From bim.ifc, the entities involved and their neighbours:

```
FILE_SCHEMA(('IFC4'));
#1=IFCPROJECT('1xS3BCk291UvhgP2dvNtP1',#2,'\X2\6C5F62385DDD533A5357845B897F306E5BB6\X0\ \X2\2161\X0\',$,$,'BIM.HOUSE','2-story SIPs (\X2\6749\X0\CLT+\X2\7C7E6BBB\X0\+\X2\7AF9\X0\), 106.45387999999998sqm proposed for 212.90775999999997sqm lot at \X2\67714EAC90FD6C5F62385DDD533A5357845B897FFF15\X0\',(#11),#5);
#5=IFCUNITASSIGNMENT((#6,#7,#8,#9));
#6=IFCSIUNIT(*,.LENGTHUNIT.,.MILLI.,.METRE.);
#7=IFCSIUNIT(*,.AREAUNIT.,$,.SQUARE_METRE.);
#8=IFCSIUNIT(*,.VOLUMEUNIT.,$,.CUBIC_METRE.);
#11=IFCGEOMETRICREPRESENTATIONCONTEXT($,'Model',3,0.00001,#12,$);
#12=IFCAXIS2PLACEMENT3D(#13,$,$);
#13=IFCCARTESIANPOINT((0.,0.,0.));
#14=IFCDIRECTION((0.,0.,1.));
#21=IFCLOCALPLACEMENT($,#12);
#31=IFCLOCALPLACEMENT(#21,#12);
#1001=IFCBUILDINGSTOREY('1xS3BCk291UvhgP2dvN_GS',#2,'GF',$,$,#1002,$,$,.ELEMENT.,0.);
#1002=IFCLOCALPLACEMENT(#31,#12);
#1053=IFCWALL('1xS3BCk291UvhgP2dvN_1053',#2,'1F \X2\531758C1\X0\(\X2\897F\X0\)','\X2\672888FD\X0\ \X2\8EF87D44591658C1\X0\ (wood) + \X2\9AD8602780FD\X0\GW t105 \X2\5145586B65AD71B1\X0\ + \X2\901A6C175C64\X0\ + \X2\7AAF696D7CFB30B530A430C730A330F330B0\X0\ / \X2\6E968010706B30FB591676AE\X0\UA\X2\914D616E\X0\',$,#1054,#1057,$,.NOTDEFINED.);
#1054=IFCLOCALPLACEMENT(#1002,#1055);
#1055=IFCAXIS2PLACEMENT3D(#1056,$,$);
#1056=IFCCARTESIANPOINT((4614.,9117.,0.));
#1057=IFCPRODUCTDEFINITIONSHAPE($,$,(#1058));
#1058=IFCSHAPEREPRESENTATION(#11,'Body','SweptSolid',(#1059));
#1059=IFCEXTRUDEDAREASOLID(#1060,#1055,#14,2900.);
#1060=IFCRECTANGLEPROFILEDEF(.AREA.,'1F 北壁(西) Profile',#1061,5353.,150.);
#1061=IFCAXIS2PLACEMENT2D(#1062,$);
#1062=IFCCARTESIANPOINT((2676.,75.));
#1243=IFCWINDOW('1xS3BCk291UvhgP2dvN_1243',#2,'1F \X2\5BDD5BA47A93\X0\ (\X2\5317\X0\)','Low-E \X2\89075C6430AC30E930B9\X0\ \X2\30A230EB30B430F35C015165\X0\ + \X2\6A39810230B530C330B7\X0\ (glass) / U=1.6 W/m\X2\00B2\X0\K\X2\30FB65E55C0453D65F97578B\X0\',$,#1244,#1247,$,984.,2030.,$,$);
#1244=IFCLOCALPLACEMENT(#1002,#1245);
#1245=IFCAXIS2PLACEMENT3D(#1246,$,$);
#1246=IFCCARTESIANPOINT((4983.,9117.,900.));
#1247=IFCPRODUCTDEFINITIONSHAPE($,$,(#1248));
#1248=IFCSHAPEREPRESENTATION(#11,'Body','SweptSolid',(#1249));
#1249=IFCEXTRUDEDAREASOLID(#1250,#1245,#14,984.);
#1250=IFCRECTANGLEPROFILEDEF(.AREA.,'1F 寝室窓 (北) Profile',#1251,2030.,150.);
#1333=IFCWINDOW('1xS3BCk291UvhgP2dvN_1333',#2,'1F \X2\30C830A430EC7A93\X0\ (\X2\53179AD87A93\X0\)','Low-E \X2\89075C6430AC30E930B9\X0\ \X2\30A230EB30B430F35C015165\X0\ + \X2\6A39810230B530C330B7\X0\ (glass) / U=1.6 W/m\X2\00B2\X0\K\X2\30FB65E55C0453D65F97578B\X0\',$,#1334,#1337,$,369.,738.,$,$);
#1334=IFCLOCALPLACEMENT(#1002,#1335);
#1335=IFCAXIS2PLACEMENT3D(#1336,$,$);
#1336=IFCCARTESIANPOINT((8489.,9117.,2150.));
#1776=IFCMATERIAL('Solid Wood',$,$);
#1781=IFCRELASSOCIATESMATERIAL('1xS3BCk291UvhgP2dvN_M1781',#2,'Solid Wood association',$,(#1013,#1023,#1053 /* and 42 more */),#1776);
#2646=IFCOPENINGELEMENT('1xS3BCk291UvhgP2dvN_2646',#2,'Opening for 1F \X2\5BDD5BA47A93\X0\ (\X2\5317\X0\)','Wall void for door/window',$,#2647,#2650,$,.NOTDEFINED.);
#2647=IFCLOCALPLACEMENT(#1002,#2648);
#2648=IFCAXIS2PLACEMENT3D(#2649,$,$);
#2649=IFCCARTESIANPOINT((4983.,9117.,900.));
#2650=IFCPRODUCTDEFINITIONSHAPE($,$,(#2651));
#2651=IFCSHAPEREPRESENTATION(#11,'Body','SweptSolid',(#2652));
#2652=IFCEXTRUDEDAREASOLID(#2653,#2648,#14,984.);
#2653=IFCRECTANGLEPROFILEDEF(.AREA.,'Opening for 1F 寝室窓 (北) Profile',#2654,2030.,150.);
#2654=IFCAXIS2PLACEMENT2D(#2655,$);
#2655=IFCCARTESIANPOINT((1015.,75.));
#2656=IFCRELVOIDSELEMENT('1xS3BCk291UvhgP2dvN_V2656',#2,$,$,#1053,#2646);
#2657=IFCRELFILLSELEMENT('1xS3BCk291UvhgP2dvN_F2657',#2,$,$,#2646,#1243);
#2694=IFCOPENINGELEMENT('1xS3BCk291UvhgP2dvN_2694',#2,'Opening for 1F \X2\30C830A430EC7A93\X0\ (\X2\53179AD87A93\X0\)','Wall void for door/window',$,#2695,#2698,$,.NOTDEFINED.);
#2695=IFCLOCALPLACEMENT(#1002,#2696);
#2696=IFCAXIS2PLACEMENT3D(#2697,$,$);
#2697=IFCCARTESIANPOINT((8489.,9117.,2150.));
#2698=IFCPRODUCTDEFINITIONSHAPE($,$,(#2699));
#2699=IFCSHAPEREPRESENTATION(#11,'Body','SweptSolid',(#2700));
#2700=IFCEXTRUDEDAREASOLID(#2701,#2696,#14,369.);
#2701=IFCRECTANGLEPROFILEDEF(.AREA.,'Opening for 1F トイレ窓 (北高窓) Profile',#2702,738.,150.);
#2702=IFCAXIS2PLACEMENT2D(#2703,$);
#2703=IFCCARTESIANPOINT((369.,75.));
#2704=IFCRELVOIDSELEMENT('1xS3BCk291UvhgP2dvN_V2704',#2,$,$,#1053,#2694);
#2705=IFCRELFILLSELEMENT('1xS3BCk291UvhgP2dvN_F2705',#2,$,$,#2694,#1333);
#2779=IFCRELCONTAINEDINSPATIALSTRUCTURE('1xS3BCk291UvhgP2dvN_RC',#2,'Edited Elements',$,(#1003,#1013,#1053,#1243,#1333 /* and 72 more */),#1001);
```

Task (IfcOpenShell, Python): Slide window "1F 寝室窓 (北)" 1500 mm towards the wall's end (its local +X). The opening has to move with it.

```python
import ifcopenshell
import ifcopenshell.api.geometry
import ifcopenshell.util.placement

model = ifcopenshell.open("bim.ifc")

window = model.by_id(1243)
opening = window.FillsVoids[0].RelatingOpeningElement
wall = opening.VoidsElements[0].RelatingBuildingElement

wall_matrix = ifcopenshell.util.placement.get_local_placement(wall.ObjectPlacement)
shift = wall_matrix[:3, 0] * 1500.0
before = ifcopenshell.util.placement.get_local_placement(window.ObjectPlacement)[:3, 3].copy()

# The window is not placed relative to its opening, so move both.
for product in (opening, window):
    matrix = ifcopenshell.util.placement.get_local_placement(product.ObjectPlacement)
    matrix[:3, 3] += shift
    ifcopenshell.api.geometry.edit_object_placement(model, product=product, matrix=matrix, is_si=False)

after = ifcopenshell.util.placement.get_local_placement(window.ObjectPlacement)[:3, 3]
print("window moved by", (after - before).round(3) + 0.0)

model.write("bim_edited.ifc")
```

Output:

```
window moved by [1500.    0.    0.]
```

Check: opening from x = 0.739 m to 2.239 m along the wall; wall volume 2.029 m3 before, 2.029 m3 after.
